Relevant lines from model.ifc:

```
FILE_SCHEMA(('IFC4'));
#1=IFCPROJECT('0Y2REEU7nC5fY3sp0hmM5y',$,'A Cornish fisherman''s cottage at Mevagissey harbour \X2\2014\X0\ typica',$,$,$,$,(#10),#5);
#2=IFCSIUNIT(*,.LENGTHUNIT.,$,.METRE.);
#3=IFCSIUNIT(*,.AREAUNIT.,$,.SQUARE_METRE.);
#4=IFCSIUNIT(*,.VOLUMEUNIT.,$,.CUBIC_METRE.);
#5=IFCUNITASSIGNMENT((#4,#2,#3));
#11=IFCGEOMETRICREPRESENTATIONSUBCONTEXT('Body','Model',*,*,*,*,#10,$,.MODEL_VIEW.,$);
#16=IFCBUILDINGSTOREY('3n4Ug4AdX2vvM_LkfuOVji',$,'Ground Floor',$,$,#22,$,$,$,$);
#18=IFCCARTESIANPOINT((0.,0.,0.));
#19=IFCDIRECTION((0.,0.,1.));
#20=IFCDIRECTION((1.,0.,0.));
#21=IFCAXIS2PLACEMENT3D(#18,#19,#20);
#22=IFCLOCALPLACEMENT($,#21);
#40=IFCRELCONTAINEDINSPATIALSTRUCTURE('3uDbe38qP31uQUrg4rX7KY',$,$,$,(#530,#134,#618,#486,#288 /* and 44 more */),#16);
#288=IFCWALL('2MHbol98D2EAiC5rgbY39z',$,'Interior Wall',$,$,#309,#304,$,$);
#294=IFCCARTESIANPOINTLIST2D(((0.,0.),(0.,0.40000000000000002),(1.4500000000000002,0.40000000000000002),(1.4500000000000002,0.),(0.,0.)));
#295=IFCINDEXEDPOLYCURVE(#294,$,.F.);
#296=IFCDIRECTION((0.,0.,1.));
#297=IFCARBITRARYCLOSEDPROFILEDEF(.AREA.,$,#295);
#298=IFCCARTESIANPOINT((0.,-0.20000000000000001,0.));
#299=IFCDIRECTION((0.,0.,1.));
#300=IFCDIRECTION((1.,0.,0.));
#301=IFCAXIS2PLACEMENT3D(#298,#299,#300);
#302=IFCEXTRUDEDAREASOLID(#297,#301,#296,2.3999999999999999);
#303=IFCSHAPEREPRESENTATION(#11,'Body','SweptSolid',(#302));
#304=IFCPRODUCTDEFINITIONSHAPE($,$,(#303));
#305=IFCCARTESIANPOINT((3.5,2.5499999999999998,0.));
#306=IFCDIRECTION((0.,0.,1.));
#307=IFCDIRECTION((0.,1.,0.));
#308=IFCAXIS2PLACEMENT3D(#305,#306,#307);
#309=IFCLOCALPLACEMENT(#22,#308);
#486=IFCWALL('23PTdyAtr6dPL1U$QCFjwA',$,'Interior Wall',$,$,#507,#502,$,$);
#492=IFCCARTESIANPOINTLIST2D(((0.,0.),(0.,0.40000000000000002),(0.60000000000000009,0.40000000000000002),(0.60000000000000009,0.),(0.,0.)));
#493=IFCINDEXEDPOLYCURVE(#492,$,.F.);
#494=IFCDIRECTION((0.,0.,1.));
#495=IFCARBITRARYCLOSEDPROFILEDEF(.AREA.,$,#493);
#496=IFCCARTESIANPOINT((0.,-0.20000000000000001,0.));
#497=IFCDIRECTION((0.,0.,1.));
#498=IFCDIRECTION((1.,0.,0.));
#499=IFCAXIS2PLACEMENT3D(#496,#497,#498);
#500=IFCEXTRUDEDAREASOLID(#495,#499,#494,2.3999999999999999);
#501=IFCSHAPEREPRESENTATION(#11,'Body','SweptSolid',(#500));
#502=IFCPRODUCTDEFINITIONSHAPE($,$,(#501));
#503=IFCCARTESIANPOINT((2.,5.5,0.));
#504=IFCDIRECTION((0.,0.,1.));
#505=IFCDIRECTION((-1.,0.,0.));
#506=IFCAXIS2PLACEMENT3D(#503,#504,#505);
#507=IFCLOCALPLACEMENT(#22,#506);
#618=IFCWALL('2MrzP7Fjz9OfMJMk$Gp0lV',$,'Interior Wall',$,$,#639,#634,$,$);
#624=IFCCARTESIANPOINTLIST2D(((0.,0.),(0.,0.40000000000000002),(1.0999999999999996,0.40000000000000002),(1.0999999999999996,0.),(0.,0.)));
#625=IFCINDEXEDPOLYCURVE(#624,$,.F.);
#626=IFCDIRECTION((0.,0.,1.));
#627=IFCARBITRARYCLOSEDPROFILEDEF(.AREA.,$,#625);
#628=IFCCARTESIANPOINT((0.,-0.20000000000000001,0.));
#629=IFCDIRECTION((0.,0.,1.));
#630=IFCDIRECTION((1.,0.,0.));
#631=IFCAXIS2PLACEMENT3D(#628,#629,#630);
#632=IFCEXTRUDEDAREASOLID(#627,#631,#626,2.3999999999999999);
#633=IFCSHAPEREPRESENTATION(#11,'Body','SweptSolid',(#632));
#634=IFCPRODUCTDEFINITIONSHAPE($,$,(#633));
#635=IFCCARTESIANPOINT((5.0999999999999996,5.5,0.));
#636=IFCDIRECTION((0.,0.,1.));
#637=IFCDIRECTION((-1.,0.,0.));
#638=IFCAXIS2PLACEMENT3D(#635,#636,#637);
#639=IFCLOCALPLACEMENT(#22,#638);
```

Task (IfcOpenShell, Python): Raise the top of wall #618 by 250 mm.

```python
import ifcopenshell
import ifcopenshell.geom
import ifcopenshell.util.representation
import ifcopenshell.util.shape
import ifcopenshell.util.unit

model = ifcopenshell.open("model.ifc")
unit_scale = ifcopenshell.util.unit.calculate_unit_scale(model)
settings = ifcopenshell.geom.settings()


def volume(element):
    """Net volume in cubic metres, openings subtracted."""
    shape = ifcopenshell.geom.create_shape(settings, element)
    return ifcopenshell.util.shape.get_volume(shape.geometry)


wall = model.by_guid("2MrzP7Fjz9OfMJMk$Gp0lV")
before = volume(wall)

body = ifcopenshell.util.representation.get_representation(wall, "Model", "Body")
solid = body.Items[0]
old_height = solid.Depth
solid.Depth += 0.25 / unit_scale
after = volume(wall)

print(f"height {old_height:g} -> {solid.Depth:g}, volume {before:.3f} -> {after:.3f} m3")

model.write("model_v2.ifc")
```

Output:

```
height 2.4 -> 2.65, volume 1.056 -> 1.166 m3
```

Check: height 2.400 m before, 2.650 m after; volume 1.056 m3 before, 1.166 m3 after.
